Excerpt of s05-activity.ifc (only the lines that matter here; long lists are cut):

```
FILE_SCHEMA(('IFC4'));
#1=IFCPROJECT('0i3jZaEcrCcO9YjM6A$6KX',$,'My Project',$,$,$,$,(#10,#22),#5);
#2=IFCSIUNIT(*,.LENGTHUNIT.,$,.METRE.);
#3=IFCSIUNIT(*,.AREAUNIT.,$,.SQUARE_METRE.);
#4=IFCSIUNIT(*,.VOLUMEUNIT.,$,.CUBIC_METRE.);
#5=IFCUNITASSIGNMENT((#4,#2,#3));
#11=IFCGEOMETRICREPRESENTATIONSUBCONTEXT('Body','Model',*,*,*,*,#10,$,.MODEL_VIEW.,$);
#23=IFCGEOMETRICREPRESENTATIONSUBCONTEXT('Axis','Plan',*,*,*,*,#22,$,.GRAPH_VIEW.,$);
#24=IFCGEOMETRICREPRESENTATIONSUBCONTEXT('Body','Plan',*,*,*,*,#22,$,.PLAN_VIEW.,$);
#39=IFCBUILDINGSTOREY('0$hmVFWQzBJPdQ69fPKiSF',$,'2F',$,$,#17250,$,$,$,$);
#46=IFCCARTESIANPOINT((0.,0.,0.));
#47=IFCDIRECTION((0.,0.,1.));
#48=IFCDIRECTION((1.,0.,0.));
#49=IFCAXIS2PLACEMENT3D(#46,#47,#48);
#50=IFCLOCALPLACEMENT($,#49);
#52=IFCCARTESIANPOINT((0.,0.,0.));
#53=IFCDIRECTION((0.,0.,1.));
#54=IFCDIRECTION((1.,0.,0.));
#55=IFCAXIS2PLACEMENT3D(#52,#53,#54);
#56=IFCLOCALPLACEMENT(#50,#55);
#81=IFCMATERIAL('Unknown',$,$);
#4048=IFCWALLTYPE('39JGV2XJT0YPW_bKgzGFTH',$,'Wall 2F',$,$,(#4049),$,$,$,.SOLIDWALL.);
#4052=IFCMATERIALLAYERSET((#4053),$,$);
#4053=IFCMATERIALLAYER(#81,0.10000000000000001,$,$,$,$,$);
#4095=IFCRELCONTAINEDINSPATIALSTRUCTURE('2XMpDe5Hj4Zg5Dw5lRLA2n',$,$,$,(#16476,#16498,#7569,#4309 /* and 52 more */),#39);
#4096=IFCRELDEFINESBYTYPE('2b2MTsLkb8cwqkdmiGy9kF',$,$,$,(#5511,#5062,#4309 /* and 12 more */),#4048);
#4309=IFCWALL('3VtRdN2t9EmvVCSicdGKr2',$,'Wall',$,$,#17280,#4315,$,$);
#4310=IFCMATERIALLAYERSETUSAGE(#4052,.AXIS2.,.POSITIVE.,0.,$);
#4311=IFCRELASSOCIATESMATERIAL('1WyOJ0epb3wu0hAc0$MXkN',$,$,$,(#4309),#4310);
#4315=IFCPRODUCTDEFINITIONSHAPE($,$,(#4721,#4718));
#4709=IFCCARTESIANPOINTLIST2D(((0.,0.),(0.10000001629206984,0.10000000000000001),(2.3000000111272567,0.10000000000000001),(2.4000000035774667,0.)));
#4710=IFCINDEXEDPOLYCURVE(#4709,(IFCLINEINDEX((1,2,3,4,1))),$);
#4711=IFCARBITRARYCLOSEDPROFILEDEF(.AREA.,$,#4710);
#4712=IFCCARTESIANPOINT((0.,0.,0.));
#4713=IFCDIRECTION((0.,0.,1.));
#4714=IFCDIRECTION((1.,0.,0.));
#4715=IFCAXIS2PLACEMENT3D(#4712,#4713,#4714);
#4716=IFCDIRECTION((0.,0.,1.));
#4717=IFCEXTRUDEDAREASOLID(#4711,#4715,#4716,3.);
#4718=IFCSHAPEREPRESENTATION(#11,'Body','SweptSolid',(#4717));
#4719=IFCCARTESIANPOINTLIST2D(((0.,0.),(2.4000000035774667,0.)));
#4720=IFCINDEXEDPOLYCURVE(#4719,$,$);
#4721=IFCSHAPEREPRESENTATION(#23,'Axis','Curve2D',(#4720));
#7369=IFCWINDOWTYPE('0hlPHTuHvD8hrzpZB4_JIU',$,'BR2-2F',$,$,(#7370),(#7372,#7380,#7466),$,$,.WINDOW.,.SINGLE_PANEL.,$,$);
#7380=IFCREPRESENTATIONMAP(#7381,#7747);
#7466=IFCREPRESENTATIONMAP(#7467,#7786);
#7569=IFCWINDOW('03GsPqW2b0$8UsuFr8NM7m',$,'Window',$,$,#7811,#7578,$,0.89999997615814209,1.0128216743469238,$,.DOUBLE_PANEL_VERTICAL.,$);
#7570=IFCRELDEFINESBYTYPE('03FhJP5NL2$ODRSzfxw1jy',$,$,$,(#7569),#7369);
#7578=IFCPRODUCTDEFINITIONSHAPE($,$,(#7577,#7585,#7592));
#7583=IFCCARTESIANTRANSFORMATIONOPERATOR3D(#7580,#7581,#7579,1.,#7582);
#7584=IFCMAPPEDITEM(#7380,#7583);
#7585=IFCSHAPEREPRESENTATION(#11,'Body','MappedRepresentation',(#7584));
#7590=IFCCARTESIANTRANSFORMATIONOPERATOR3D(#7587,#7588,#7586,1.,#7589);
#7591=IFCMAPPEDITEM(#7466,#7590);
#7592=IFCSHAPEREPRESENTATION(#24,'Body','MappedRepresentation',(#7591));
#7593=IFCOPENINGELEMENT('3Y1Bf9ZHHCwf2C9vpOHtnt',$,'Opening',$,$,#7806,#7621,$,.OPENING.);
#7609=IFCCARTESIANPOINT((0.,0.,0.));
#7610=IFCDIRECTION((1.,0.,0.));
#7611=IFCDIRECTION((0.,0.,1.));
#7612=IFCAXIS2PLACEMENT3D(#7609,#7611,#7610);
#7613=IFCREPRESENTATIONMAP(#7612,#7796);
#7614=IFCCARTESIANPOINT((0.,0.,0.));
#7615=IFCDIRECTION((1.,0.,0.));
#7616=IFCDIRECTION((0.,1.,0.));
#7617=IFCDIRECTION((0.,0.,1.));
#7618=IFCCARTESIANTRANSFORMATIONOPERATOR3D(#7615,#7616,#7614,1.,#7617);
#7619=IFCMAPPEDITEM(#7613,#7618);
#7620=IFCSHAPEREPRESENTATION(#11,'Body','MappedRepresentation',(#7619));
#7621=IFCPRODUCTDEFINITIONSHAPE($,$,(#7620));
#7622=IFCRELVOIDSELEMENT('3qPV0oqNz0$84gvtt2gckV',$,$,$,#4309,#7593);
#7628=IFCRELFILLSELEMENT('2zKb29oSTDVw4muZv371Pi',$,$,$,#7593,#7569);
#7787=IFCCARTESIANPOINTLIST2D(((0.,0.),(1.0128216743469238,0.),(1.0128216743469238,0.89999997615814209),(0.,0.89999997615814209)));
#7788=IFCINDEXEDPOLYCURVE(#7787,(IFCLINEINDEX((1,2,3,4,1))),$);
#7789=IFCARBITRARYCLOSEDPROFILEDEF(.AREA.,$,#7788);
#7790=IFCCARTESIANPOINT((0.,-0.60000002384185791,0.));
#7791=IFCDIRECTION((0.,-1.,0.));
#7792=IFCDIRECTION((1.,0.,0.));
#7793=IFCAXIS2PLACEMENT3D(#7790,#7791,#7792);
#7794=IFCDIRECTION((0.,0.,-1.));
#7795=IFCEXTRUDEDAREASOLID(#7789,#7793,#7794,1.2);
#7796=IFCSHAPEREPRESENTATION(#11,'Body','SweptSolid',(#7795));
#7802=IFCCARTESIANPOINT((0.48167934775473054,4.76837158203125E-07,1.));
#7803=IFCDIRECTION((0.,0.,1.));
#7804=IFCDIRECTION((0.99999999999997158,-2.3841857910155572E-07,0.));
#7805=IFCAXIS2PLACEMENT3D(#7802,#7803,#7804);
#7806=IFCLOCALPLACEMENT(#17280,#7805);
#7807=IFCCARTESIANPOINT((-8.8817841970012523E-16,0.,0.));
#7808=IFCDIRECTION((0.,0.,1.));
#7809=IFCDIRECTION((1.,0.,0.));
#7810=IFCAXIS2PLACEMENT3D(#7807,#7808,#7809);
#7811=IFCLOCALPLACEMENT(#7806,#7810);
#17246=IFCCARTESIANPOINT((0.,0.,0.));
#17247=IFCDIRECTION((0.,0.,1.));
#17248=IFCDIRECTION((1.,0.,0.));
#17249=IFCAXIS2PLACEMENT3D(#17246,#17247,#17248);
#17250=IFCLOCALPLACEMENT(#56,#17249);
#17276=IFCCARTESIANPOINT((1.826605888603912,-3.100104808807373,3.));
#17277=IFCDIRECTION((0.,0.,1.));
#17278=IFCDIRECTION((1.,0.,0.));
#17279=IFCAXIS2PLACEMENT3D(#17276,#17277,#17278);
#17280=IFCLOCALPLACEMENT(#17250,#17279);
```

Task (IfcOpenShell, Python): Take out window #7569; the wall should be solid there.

```python
import ifcopenshell
import ifcopenshell.api.feature
import ifcopenshell.api.root
import ifcopenshell.geom
import ifcopenshell.util.shape

model = ifcopenshell.open("s05-activity.ifc")
settings = ifcopenshell.geom.settings()


def volume(element):
    """Net volume in cubic metres, openings subtracted."""
    shape = ifcopenshell.geom.create_shape(settings, element)
    return ifcopenshell.util.shape.get_volume(shape.geometry)


window = model.by_id(7569)
opening = window.FillsVoids[0].RelatingOpeningElement
wall = opening.VoidsElements[0].RelatingBuildingElement
before = volume(wall)

ifcopenshell.api.root.remove_product(model, product=window)
ifcopenshell.api.feature.remove_feature(model, feature=opening)

after = volume(wall)

print(f"wall volume {before:.3f} -> {after:.3f} m3")

model.write("s05-activity_updated.ifc")
```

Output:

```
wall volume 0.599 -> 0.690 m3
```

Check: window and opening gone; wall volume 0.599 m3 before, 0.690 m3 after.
